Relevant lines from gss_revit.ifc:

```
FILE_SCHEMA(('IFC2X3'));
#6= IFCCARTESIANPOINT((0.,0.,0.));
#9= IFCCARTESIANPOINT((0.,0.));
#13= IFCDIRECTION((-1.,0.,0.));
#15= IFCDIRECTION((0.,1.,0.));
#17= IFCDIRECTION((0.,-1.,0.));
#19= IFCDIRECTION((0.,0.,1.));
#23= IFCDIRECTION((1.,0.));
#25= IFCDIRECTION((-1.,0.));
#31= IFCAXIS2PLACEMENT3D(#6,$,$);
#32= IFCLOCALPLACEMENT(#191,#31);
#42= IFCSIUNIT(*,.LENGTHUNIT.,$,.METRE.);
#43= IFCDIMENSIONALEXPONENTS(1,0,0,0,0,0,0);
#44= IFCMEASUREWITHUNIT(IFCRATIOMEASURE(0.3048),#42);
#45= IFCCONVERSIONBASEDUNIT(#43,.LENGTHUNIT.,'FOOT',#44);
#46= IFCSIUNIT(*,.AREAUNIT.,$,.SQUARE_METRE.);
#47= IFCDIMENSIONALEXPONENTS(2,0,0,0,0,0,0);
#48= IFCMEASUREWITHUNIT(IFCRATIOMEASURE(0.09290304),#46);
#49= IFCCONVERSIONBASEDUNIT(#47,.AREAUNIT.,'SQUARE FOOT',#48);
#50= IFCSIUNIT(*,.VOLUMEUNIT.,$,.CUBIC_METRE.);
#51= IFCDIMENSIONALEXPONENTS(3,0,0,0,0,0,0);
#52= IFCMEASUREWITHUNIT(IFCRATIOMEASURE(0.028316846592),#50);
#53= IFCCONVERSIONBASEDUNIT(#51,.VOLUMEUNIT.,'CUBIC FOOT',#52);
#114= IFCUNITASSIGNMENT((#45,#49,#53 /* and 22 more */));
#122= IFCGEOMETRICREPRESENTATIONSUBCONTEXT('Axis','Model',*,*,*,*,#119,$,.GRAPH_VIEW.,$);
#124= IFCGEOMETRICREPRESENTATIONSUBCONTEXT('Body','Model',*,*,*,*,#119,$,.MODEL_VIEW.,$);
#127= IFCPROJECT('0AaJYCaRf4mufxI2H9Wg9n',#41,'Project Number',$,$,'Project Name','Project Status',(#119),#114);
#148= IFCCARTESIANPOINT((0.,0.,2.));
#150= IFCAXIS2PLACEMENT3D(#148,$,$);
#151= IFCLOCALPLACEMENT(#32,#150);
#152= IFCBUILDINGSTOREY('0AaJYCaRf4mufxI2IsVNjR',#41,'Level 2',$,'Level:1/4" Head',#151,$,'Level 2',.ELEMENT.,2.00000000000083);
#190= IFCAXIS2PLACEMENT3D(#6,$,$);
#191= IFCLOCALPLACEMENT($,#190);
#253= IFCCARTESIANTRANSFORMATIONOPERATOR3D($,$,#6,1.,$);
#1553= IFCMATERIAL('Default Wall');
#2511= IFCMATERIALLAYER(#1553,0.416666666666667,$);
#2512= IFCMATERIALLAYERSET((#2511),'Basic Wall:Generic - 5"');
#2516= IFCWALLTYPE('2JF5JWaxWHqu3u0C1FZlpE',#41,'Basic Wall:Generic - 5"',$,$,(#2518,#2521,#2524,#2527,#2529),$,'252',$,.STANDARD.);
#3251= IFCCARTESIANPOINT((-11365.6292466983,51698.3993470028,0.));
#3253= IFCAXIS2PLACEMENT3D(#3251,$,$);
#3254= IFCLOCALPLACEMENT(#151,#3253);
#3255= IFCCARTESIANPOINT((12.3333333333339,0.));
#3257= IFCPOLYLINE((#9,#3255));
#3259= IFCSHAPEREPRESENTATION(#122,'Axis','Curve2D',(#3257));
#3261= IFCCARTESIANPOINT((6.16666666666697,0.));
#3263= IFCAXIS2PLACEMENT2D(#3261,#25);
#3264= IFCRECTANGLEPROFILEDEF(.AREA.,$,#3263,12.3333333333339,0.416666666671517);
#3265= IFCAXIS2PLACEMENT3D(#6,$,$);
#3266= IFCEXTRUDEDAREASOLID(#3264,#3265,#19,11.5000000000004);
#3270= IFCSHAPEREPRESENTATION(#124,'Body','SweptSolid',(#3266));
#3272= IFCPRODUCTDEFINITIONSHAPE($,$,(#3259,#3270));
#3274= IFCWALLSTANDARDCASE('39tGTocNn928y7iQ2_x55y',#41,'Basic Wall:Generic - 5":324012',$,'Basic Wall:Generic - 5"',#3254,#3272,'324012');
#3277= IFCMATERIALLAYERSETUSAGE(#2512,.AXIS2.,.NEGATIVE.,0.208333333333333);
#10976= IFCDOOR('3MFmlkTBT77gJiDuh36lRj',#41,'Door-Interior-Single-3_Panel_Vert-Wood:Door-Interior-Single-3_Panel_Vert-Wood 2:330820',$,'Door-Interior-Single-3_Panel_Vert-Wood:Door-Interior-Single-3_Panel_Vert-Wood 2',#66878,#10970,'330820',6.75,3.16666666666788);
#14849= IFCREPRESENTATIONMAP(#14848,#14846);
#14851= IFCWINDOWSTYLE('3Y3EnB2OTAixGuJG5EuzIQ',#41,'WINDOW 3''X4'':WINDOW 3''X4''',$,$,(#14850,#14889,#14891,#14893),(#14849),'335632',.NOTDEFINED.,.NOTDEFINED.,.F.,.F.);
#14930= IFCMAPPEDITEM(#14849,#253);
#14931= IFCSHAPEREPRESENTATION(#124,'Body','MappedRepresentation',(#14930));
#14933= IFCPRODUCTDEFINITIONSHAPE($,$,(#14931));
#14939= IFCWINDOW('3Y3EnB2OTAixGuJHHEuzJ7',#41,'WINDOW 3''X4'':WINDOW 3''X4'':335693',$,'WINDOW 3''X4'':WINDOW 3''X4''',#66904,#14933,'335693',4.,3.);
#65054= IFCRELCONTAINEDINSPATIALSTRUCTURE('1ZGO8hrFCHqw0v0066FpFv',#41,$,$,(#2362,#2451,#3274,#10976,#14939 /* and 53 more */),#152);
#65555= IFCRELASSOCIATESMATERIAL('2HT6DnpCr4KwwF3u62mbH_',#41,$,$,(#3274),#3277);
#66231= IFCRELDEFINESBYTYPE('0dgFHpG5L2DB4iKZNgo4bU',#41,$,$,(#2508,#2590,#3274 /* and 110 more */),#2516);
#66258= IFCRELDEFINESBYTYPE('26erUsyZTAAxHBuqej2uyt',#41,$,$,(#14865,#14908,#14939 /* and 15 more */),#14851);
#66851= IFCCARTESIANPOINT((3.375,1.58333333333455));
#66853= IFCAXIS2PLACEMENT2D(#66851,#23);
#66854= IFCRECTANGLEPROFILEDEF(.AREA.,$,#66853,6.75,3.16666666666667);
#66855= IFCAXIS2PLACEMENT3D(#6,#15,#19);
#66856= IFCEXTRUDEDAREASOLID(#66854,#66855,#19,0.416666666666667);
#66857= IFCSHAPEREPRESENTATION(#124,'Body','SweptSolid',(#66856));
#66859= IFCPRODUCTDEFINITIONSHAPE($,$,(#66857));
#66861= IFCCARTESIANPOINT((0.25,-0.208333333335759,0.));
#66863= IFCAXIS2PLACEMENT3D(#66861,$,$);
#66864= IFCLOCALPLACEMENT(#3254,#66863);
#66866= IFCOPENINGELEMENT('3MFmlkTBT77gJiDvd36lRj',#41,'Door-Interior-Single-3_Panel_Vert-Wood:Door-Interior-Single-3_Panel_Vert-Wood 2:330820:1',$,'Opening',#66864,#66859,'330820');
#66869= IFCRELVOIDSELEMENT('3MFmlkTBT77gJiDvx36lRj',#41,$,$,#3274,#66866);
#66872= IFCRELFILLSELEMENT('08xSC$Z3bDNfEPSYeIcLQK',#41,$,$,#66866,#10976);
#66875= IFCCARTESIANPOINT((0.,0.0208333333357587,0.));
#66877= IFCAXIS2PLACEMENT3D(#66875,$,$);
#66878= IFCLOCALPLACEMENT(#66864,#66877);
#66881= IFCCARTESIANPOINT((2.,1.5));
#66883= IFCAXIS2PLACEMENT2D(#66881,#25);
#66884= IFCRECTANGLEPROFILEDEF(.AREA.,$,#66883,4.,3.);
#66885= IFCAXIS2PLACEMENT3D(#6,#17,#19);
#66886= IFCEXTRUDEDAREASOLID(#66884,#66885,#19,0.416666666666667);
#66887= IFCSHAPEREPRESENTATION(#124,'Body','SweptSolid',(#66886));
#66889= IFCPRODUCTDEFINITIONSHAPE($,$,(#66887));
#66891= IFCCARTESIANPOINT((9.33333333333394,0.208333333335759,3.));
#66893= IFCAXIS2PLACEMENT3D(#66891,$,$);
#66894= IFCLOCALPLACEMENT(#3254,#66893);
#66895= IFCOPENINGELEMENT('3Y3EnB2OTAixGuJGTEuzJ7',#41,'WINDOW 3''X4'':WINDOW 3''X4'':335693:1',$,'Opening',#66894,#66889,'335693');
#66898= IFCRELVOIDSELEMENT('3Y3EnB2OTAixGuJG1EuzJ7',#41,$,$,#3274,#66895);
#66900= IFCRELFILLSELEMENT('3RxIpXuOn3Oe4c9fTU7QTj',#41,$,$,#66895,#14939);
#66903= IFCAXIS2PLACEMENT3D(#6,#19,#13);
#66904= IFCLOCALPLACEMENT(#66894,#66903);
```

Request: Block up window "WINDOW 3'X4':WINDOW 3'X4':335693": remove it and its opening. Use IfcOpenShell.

```python
import ifcopenshell
import ifcopenshell.api.feature
import ifcopenshell.api.root
import ifcopenshell.geom
import ifcopenshell.util.shape

model = ifcopenshell.open("gss_revit.ifc")
settings = ifcopenshell.geom.settings()


def volume(element):
    """Net volume in cubic metres, openings subtracted."""
    shape = ifcopenshell.geom.create_shape(settings, element)
    return ifcopenshell.util.shape.get_volume(shape.geometry)


window = model.by_guid("3Y3EnB2OTAixGuJHHEuzJ7")
opening = window.FillsVoids[0].RelatingOpeningElement
wall = opening.VoidsElements[0].RelatingBuildingElement
before = volume(wall)

ifcopenshell.api.root.remove_product(model, product=window)
ifcopenshell.api.feature.remove_feature(model, feature=opening)

after = volume(wall)

print(f"wall volume {before:.3f} -> {after:.3f} m3")

model.write("gss_revit_edited.ifc")
```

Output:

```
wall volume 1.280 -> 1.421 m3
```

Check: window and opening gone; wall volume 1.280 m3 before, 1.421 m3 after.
